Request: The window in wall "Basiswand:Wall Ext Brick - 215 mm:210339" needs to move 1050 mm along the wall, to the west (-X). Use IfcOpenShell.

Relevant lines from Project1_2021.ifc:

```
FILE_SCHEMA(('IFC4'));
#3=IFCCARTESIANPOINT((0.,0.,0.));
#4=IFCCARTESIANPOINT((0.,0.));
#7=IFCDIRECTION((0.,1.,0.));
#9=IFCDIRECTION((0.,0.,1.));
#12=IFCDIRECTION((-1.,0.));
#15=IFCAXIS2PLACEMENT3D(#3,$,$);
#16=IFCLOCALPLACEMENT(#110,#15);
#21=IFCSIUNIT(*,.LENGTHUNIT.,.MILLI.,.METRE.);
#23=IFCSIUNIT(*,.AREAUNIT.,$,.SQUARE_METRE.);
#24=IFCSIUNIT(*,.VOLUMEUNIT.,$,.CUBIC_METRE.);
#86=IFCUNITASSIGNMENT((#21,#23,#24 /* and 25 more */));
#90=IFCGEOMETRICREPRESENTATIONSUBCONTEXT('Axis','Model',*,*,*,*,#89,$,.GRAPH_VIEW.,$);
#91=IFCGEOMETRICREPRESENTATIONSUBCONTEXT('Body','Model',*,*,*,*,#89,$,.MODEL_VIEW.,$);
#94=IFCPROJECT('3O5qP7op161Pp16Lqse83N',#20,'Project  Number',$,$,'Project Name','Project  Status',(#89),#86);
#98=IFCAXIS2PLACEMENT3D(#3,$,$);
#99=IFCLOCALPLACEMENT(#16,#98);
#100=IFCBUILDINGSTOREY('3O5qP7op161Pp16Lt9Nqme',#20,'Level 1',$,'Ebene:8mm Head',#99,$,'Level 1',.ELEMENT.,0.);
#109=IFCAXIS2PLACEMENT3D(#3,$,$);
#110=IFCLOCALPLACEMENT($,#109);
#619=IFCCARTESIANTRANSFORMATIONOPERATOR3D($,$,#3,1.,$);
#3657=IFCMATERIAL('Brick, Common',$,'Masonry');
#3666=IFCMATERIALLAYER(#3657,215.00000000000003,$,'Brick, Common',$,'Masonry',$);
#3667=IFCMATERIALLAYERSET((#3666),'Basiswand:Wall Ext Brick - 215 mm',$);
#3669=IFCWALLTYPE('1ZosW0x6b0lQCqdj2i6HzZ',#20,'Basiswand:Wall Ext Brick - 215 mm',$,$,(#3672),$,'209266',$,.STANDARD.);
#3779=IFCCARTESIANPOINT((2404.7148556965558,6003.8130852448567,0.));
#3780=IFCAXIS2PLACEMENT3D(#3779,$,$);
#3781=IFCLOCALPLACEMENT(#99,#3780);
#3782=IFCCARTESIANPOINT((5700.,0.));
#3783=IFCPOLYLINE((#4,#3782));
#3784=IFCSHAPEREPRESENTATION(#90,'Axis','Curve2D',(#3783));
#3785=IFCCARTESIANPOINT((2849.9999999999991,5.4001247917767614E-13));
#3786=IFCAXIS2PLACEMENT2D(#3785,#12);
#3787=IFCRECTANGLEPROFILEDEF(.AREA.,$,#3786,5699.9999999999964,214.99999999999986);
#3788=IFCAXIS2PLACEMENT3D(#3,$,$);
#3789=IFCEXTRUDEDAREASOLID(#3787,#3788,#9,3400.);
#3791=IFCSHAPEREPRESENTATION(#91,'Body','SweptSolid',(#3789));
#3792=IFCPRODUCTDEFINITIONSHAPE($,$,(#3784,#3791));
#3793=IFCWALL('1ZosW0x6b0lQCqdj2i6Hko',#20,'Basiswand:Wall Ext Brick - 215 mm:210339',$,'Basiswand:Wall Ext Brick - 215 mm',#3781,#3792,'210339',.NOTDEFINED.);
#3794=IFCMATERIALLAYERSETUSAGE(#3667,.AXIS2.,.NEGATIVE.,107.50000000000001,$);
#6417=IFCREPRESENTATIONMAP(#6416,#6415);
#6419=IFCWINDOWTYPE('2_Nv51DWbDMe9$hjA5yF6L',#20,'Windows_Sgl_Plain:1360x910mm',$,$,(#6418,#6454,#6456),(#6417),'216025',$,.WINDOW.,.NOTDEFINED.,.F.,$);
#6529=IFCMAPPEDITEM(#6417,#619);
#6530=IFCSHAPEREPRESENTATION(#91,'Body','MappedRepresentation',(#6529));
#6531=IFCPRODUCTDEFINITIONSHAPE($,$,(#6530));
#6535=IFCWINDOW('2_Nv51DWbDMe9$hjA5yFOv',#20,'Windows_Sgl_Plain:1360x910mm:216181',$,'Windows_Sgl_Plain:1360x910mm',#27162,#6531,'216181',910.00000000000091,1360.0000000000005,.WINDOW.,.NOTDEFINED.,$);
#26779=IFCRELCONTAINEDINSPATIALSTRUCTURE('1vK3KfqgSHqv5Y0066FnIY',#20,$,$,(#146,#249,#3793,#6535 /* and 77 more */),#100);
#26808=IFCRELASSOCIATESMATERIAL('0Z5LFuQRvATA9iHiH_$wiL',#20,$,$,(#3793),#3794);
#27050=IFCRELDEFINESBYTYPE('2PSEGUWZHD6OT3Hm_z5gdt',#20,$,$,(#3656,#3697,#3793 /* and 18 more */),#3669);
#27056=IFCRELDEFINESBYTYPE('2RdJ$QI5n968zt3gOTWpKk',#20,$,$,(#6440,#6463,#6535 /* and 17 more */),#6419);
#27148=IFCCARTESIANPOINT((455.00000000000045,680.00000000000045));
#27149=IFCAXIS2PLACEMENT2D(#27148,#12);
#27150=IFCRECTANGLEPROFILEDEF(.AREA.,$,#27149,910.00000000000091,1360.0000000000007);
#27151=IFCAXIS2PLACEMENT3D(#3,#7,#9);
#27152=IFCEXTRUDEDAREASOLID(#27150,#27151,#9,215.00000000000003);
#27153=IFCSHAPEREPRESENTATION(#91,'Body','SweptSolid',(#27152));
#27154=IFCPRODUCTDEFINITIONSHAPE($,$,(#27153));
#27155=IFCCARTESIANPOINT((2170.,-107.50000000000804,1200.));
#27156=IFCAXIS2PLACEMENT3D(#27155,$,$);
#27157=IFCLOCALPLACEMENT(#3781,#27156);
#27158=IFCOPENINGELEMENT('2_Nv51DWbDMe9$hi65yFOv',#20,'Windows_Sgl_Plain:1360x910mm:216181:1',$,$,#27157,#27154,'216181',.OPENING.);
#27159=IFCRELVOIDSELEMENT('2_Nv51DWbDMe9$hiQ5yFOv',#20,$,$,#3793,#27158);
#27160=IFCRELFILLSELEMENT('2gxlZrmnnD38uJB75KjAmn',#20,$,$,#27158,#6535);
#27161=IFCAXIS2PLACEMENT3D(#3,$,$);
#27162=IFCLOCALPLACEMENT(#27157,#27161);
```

```python
import ifcopenshell
import ifcopenshell.api.geometry
import ifcopenshell.util.placement

model = ifcopenshell.open("Project1_2021.ifc")

window = model.by_guid("2_Nv51DWbDMe9$hjA5yFOv")
opening = window.FillsVoids[0].RelatingOpeningElement
wall = opening.VoidsElements[0].RelatingBuildingElement

wall_matrix = ifcopenshell.util.placement.get_local_placement(wall.ObjectPlacement)
shift = wall_matrix[:3, 0] * -1050.0
before = ifcopenshell.util.placement.get_local_placement(window.ObjectPlacement)[:3, 3].copy()

# The window is placed relative to its opening, so it follows when the opening moves.
matrix = ifcopenshell.util.placement.get_local_placement(opening.ObjectPlacement)
matrix[:3, 3] += shift
ifcopenshell.api.geometry.edit_object_placement(
    model, product=opening, matrix=matrix, is_si=False, should_transform_children=True
)

after = ifcopenshell.util.placement.get_local_placement(window.ObjectPlacement)[:3, 3]
print("window moved by", (after - before).round(3) + 0.0)

model.write("Project1_2021_v2.ifc")
```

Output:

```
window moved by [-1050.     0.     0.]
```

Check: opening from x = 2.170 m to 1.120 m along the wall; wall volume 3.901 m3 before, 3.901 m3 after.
